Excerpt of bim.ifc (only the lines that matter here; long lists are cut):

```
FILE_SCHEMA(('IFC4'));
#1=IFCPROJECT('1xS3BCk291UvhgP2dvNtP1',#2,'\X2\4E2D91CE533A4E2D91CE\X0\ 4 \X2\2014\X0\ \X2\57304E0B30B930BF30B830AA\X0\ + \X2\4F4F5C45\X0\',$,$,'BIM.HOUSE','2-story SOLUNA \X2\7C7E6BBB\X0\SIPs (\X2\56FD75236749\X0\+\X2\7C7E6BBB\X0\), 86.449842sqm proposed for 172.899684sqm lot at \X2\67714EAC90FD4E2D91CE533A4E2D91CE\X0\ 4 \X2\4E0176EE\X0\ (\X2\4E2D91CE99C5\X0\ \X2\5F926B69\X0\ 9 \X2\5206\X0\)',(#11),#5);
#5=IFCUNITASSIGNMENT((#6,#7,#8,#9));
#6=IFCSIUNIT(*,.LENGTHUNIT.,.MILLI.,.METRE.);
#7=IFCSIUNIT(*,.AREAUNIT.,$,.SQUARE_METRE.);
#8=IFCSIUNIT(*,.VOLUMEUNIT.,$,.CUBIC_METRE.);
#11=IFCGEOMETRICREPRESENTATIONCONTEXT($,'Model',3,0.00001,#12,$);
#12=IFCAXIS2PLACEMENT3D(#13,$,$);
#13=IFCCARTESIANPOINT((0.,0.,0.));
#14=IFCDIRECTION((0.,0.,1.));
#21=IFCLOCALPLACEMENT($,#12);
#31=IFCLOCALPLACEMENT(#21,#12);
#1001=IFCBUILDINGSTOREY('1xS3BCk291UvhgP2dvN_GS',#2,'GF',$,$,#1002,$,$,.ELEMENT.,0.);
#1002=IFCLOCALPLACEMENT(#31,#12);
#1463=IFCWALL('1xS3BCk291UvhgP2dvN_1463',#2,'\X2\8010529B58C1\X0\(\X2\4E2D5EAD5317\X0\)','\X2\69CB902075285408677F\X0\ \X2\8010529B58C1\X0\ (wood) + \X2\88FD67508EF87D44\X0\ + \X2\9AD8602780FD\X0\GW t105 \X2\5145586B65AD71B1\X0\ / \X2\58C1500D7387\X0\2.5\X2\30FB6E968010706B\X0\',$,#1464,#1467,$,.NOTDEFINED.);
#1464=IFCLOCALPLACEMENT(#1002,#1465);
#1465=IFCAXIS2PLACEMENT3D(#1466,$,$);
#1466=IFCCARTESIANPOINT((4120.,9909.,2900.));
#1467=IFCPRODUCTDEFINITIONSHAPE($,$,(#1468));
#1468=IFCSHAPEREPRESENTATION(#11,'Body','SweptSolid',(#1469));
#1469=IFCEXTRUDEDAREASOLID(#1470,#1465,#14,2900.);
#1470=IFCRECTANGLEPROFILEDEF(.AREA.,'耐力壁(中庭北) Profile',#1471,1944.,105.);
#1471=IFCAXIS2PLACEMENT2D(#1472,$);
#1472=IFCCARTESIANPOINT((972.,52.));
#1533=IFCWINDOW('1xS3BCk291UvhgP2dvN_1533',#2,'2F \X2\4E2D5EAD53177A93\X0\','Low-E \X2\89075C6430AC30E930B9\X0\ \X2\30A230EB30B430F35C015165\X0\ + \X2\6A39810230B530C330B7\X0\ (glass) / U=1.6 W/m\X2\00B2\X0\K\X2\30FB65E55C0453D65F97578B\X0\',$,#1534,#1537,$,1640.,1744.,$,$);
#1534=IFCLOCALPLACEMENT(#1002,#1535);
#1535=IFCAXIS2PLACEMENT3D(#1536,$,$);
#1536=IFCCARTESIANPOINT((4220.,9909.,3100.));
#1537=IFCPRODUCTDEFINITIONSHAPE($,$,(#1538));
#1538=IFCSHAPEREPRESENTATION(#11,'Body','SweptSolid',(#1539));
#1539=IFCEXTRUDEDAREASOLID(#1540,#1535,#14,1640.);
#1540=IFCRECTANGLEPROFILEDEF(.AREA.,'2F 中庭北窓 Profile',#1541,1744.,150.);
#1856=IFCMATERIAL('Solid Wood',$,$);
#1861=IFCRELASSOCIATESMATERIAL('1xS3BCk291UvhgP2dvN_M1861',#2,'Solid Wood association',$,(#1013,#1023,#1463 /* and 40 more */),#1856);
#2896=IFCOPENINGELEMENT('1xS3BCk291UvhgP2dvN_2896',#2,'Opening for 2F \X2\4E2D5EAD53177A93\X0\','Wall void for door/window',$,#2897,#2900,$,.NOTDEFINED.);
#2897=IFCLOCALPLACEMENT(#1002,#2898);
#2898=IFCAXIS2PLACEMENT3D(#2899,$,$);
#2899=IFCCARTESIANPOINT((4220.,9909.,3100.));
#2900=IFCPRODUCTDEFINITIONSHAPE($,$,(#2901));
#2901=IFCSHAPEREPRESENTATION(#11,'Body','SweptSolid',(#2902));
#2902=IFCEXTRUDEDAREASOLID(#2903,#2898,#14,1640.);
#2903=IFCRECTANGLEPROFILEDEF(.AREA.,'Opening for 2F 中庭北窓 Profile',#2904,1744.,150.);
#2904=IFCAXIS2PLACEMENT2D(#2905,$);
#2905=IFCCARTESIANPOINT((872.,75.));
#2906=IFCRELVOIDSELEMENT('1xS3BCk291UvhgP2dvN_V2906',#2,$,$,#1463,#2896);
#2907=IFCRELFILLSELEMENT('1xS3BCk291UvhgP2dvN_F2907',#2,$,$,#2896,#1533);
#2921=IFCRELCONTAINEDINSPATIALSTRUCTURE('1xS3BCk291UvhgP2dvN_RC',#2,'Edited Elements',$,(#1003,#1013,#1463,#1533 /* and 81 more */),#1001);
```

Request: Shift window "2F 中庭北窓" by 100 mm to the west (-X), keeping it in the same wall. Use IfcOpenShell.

```python
import ifcopenshell
import ifcopenshell.api.geometry
import ifcopenshell.util.placement
import ifcopenshell.util.unit

model = ifcopenshell.open("bim.ifc")
unit_scale = ifcopenshell.util.unit.calculate_unit_scale(model)

window = model.by_id(1533)
opening = window.FillsVoids[0].RelatingOpeningElement
wall = opening.VoidsElements[0].RelatingBuildingElement

wall_matrix = ifcopenshell.util.placement.get_local_placement(wall.ObjectPlacement)
shift = wall_matrix[:3, 0] * -0.1 / unit_scale
before = ifcopenshell.util.placement.get_local_placement(window.ObjectPlacement)[:3, 3].copy()

# The window is not placed relative to its opening, so move both.
for product in (opening, window):
    matrix = ifcopenshell.util.placement.get_local_placement(product.ObjectPlacement)
    matrix[:3, 3] += shift
    ifcopenshell.api.geometry.edit_object_placement(model, product=product, matrix=matrix, is_si=False)

after = ifcopenshell.util.placement.get_local_placement(window.ObjectPlacement)[:3, 3]
print("window moved by", (after - before).round(3) + 0.0)

model.write("bim_rev.ifc")
```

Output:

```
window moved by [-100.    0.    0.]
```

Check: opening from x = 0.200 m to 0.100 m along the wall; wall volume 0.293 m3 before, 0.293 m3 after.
